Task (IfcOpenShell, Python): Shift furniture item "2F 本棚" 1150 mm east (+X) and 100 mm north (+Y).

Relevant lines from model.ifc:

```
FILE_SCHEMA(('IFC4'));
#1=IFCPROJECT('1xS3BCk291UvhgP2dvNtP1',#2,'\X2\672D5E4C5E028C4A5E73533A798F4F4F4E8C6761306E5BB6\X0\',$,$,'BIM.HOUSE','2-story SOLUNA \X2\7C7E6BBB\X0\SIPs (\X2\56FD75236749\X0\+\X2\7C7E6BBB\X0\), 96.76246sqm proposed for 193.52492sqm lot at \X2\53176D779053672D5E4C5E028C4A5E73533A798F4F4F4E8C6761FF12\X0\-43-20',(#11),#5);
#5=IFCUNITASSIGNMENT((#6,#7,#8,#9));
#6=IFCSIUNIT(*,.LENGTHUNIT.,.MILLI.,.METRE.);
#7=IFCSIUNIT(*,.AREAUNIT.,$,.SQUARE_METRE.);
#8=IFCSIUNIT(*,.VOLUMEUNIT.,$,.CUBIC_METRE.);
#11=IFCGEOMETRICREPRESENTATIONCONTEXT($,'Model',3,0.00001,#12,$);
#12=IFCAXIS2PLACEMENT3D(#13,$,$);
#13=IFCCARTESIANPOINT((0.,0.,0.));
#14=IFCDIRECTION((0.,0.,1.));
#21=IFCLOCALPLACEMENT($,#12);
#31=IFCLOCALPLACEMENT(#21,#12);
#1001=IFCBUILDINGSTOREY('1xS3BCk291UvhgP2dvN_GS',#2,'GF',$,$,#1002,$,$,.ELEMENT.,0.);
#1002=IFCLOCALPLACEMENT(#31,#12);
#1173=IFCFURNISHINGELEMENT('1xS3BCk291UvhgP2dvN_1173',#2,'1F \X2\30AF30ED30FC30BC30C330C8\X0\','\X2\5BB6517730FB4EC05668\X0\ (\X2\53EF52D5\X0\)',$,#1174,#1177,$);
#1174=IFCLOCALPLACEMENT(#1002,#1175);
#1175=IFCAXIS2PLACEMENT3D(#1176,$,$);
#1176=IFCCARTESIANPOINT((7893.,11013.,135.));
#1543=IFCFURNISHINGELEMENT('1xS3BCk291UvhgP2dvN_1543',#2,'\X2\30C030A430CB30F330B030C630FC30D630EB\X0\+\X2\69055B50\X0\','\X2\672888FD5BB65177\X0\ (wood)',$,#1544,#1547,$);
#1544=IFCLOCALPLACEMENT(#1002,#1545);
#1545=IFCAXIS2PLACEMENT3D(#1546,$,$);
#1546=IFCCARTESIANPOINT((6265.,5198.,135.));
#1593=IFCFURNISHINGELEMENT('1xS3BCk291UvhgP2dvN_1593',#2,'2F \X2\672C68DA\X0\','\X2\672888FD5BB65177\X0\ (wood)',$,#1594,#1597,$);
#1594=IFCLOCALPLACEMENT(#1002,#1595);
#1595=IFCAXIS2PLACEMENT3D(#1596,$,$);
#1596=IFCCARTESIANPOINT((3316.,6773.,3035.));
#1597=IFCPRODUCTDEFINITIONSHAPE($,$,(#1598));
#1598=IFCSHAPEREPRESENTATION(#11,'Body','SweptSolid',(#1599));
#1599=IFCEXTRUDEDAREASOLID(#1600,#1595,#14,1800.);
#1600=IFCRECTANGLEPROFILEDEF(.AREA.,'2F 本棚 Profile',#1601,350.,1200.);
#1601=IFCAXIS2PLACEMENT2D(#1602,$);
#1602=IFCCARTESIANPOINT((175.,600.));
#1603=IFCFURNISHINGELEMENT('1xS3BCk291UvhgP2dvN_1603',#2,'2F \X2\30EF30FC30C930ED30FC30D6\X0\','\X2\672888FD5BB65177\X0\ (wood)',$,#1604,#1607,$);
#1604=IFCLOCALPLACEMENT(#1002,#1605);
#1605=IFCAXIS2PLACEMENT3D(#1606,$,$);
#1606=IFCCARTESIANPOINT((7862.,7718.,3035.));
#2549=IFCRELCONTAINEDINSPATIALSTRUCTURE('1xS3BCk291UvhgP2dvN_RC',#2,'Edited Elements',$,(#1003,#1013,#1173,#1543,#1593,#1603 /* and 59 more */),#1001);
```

```python
import ifcopenshell
import ifcopenshell.api.geometry
import ifcopenshell.util.placement

model = ifcopenshell.open("model.ifc")

item = model.by_guid("1xS3BCk291UvhgP2dvN_1593")
matrix = ifcopenshell.util.placement.get_local_placement(item.ObjectPlacement)
matrix[0, 3] += 1150.0
matrix[1, 3] += 100.0
ifcopenshell.api.geometry.edit_object_placement(model, product=item, matrix=matrix, is_si=False)

print(ifcopenshell.util.placement.get_local_placement(item.ObjectPlacement).round(3) + 0.0)

model.write("model-out.ifc")
```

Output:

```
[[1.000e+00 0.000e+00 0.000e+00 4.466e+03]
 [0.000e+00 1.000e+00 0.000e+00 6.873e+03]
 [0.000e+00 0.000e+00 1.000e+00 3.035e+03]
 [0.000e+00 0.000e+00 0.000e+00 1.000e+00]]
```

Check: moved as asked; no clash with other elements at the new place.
